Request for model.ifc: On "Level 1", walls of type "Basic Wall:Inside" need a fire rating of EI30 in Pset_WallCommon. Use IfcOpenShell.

First a look at what the model holds.

```python
import ifcopenshell
import ifcopenshell.util.element

model = ifcopenshell.open("model.ifc")
print(model.schema)
storey = next(s for s in model.by_type("IfcBuildingStorey") if s.Name == "Level 1")
walls = [e for e in ifcopenshell.util.element.get_decomposition(storey) if e.is_a("IfcWall")]
seen = {}
for e in walls:
    element_type = ifcopenshell.util.element.get_type(e)
    key = (element_type.Name if element_type != e and element_type else None, ifcopenshell.util.element.get_pset(e, "Pset_WallCommon", "FireRating"))
    seen[key] = seen.get(key, 0) + 1
for (name, value), count in sorted(seen.items(), key=str):
    print(count, "x", name, "|", value)
```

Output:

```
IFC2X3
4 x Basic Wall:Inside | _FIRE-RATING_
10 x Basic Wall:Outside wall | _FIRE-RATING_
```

```python
import ifcopenshell
import ifcopenshell.api.pset
import ifcopenshell.util.element

model = ifcopenshell.open("model.ifc")

storey = next(s for s in model.by_type("IfcBuildingStorey") if s.Name == "Level 1")
walls = [e for e in ifcopenshell.util.element.get_decomposition(storey) if e.is_a("IfcWall")]

count = 0
for e in walls:
    element_type = ifcopenshell.util.element.get_type(e)
    if element_type in (None, e) or element_type.Name != "Basic Wall:Inside":
        continue
    # add_pset returns the element's existing set when there is one.
    pset = ifcopenshell.api.pset.add_pset(model, product=e, name="Pset_WallCommon")
    ifcopenshell.api.pset.edit_pset(model, pset=pset, properties={"FireRating": "EI30"})
    count += 1

print(count, "walls updated")

model.write("model_edited.ifc")
```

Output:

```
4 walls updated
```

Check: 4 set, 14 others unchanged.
